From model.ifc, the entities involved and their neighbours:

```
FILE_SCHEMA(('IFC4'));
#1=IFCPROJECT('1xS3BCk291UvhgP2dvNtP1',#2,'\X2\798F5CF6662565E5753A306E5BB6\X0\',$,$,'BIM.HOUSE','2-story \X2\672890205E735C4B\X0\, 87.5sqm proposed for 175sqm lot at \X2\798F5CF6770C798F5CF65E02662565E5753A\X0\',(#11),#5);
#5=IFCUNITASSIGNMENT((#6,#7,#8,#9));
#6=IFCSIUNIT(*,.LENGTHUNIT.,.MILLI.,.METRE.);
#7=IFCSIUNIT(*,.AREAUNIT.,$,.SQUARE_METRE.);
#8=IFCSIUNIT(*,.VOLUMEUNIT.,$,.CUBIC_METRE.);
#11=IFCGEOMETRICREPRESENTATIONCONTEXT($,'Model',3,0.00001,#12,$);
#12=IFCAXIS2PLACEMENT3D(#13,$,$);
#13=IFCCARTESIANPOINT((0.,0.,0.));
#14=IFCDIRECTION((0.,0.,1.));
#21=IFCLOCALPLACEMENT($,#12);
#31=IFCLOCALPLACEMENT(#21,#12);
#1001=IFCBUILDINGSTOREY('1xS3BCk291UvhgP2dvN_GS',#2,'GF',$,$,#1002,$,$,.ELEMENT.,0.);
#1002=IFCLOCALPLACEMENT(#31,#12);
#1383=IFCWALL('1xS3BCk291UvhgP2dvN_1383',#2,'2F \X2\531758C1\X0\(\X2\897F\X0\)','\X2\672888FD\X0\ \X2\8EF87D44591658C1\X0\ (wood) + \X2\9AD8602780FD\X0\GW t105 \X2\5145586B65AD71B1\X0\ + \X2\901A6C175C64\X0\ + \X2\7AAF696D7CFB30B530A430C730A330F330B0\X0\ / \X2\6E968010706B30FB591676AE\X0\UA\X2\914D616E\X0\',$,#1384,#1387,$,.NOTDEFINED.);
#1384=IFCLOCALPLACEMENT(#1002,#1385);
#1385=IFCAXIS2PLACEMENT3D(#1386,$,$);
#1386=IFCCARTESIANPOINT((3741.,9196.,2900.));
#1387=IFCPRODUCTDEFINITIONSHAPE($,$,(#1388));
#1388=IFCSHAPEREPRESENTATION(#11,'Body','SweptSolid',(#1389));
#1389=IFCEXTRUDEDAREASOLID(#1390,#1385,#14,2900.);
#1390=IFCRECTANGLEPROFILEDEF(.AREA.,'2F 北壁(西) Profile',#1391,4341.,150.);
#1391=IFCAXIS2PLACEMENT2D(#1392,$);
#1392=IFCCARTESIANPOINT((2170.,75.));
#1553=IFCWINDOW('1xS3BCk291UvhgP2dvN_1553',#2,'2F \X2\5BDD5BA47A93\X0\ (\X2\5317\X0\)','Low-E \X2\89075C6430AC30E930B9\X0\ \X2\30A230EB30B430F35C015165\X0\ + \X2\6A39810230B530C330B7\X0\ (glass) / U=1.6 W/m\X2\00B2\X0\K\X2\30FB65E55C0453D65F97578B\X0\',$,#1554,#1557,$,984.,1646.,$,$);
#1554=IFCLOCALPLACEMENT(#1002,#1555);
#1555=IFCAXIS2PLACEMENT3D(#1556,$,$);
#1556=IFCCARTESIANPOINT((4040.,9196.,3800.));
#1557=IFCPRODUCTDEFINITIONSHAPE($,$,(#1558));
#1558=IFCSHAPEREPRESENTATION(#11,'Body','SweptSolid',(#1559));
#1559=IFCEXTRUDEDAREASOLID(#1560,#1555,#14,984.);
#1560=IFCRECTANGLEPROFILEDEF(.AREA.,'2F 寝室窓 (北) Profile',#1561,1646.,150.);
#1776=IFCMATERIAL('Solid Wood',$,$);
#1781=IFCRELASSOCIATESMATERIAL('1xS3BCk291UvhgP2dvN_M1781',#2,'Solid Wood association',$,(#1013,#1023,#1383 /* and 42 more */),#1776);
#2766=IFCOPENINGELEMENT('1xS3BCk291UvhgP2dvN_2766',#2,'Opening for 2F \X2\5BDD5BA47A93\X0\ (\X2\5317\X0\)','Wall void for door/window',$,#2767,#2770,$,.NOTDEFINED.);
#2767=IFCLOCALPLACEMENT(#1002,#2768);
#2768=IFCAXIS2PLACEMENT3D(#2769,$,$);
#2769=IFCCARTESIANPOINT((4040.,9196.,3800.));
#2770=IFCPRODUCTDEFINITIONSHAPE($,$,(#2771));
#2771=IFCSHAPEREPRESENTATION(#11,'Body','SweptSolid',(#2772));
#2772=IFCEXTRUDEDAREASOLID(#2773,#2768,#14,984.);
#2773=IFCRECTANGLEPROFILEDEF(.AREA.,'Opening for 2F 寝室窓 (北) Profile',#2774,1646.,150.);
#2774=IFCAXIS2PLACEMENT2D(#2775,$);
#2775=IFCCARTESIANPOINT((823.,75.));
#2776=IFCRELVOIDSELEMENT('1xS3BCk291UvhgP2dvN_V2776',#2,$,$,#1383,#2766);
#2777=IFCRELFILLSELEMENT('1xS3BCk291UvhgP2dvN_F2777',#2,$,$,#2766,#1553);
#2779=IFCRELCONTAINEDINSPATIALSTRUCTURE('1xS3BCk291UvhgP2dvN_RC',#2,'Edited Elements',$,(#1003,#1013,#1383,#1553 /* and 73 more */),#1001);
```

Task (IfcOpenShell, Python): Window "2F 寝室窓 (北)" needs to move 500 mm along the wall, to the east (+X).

```python
import ifcopenshell
import ifcopenshell.api.geometry
import ifcopenshell.util.placement
import ifcopenshell.util.unit

model = ifcopenshell.open("model.ifc")
unit_scale = ifcopenshell.util.unit.calculate_unit_scale(model)

window = model.by_guid("1xS3BCk291UvhgP2dvN_1553")
opening = window.FillsVoids[0].RelatingOpeningElement
wall = opening.VoidsElements[0].RelatingBuildingElement

wall_matrix = ifcopenshell.util.placement.get_local_placement(wall.ObjectPlacement)
shift = wall_matrix[:3, 0] * 0.5 / unit_scale
before = ifcopenshell.util.placement.get_local_placement(window.ObjectPlacement)[:3, 3].copy()

# The window is not placed relative to its opening, so move both.
for product in (opening, window):
    matrix = ifcopenshell.util.placement.get_local_placement(product.ObjectPlacement)
    matrix[:3, 3] += shift
    ifcopenshell.api.geometry.edit_object_placement(model, product=product, matrix=matrix, is_si=False)

after = ifcopenshell.util.placement.get_local_placement(window.ObjectPlacement)[:3, 3]
print("window moved by", (after - before).round(3) + 0.0)

model.write("model_v2.ifc")
```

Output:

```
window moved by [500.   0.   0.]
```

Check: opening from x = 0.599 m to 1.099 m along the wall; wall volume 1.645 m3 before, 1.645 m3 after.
